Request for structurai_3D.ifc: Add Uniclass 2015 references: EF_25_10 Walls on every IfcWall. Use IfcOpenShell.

First a look at what the model holds.

```python
import ifcopenshell

model = ifcopenshell.open("structurai_3D.ifc")
print(model.schema)
print("classifications:", [c.Name for c in model.by_type("IfcClassification")])
for ifc_class in ("IfcDoor", "IfcRoof", "IfcStair", "IfcWall", "IfcWindow"):
    print(ifc_class, len(model.by_type(ifc_class)))
```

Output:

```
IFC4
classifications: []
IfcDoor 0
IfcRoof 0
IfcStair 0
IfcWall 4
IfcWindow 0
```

```python
import ifcopenshell
import ifcopenshell.api.classification

model = ifcopenshell.open("structurai_3D.ifc")

system = ifcopenshell.api.classification.add_classification(model, classification="Uniclass 2015")

codes = {
    "IfcWall": ("EF_25_10", "Walls"),
}
for ifc_class, (code, name) in codes.items():
    products = model.by_type(ifc_class)
    ifcopenshell.api.classification.add_reference(
        model, products=products, classification=system, identification=code, name=name
    )
    print(code, len(products))

model.write("structurai_3D_rev.ifc")
```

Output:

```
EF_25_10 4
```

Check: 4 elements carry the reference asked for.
